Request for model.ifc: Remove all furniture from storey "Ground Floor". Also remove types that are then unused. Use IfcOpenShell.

First a look at what the model holds.

```python
import ifcopenshell
import ifcopenshell.util.element

model = ifcopenshell.open("model.ifc")
print(model.schema)
storey = next(s for s in model.by_type("IfcBuildingStorey") if s.Name == "Ground Floor")
furniture = [e for e in ifcopenshell.util.element.get_decomposition(storey) if e.is_a("IfcFurnishingElement")]
seen = {}
for e in furniture:
    element_type = ifcopenshell.util.element.get_type(e)
    name = element_type.Name if element_type not in (None, e) else None
    seen[name] = seen.get(name, 0) + 1
for name, count in sorted(seen.items(), key=str):
    print(count, "x", name)
```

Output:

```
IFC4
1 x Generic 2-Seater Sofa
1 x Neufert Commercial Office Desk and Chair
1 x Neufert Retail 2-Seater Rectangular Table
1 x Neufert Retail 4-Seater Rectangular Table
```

```python
import ifcopenshell
import ifcopenshell.api.root
import ifcopenshell.util.element

model = ifcopenshell.open("model.ifc")

storey = next(s for s in model.by_type("IfcBuildingStorey") if s.Name == "Ground Floor")
furniture = [e for e in ifcopenshell.util.element.get_decomposition(storey) if e.is_a("IfcFurnishingElement")]
types = {ifcopenshell.util.element.get_type(e) for e in furniture} - {None, *furniture}

for e in furniture:
    ifcopenshell.api.root.remove_product(model, product=e)
print(len(furniture), "removed")

unused = [t for t in types if not ifcopenshell.util.element.get_types(t)]
for t in unused:
    ifcopenshell.api.root.remove_product(model, product=t)
print(len(unused), "unused types removed")

model.write("model_edited.ifc")
```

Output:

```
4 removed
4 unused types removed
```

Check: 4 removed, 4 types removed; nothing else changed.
